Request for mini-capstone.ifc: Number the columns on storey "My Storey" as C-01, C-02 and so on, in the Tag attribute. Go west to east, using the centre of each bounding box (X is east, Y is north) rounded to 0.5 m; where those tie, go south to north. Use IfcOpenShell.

First a look at what the model holds.

```python
import ifcopenshell
import ifcopenshell.util.element
import ifcopenshell.util.placement

model = ifcopenshell.open("mini-capstone.ifc")
print(model.schema)
storey = next(s for s in model.by_type("IfcBuildingStorey") if s.Name == "My Storey")
columns = [e for e in ifcopenshell.util.element.get_decomposition(storey) if e.is_a("IfcColumn")]
for e in sorted(columns, key=lambda e: e.id()):
    origin = ifcopenshell.util.placement.get_local_placement(e.ObjectPlacement)[:3, 3]
    print(e.id(), e.Tag, e.Name, origin.round(2) + 0.0, sep=" | ")
```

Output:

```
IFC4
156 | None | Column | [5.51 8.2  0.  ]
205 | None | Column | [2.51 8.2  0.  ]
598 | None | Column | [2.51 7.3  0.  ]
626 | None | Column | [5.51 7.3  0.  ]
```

```python
import ifcopenshell
import ifcopenshell.geom
import ifcopenshell.util.element
import ifcopenshell.util.shape

model = ifcopenshell.open("mini-capstone.ifc")
settings = ifcopenshell.geom.settings()
settings.set("use-world-coords", True)


def centre(element):
    shape = ifcopenshell.geom.create_shape(settings, element)
    return ifcopenshell.util.shape.get_bbox_centroid(shape.geometry)


storey = next(s for s in model.by_type("IfcBuildingStorey") if s.Name == "My Storey")
columns = [e for e in ifcopenshell.util.element.get_decomposition(storey) if e.is_a("IfcColumn")]

# Insertion points can sit at a corner or the storey origin, so sort by the geometry (in metres).
centres = {e: centre(e) for e in columns}
columns.sort(key=lambda e: (round(centres[e][0] / 0.5), centres[e][1]))

for i, e in enumerate(columns, start=1):
    number = f"C-{i:02d}"
    e.Tag = number
    print(e.id(), number)

model.write("mini-capstone_updated.ifc")
```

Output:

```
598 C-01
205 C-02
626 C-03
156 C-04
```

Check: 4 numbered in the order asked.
